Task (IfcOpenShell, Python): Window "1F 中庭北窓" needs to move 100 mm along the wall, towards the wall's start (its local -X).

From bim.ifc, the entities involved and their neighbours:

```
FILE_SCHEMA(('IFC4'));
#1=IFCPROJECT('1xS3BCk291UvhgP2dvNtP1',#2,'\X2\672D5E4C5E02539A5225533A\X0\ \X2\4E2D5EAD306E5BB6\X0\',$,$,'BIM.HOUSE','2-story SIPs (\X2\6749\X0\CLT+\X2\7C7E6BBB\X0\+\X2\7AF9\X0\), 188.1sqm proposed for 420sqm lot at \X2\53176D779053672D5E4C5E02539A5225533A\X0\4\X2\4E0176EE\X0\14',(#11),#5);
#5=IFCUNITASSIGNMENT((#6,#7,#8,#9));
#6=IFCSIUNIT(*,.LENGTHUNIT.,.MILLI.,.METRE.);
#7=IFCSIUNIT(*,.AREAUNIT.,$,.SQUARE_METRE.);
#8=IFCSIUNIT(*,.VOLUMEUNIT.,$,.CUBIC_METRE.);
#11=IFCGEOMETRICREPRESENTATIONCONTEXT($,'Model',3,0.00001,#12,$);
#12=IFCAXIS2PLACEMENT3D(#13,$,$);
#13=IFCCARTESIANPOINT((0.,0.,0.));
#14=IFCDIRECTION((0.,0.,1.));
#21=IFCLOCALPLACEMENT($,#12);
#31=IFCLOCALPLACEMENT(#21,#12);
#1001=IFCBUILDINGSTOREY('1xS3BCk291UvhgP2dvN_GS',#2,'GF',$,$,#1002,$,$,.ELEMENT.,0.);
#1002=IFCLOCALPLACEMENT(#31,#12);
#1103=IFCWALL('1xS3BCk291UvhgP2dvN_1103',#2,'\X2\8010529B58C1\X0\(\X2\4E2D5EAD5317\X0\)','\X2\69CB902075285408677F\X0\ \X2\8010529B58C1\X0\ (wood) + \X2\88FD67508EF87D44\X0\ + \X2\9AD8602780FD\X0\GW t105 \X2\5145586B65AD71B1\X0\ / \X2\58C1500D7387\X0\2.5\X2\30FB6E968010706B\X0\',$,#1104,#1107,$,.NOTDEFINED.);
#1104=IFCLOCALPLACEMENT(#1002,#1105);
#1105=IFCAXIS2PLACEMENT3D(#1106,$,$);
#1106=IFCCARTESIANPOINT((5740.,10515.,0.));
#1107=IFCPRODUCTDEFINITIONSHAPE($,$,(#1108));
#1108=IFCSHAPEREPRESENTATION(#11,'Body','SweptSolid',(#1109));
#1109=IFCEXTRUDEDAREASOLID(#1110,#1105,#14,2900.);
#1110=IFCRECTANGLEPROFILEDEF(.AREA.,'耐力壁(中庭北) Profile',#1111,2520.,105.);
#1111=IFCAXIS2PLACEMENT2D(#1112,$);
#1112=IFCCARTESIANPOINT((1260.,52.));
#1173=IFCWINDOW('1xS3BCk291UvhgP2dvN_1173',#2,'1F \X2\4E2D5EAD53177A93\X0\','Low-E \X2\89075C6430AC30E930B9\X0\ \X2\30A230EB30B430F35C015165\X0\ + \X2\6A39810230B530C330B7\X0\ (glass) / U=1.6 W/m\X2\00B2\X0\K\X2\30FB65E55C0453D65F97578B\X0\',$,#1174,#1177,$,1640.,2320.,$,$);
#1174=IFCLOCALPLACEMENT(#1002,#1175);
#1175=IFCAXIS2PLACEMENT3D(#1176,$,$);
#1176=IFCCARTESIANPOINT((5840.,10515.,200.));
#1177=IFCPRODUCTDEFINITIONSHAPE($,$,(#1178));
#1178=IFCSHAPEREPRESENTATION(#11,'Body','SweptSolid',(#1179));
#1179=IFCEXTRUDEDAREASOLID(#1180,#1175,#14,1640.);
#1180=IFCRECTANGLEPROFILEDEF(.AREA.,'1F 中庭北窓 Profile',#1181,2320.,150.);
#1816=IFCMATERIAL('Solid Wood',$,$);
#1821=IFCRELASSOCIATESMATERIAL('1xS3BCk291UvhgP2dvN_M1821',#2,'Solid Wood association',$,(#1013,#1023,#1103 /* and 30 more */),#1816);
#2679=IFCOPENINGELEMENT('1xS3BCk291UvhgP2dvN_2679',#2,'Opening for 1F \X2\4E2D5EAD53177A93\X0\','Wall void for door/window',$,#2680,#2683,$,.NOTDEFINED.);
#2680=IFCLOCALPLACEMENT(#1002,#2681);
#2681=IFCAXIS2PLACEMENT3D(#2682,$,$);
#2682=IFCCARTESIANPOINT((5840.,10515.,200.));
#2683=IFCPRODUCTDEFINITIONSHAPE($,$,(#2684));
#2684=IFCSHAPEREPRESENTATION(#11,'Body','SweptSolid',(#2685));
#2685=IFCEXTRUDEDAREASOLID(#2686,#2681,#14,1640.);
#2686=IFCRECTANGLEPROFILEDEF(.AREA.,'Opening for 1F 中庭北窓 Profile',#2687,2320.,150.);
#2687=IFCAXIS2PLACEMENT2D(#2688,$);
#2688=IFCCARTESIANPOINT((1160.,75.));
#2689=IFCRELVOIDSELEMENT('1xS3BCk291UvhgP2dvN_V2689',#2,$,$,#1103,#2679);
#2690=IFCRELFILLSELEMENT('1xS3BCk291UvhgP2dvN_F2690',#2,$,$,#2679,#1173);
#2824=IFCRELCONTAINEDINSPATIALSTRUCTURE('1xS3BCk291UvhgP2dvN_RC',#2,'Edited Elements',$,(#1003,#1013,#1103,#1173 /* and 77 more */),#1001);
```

```python
import ifcopenshell
import ifcopenshell.api.geometry
import ifcopenshell.util.placement

model = ifcopenshell.open("bim.ifc")

window = model.by_guid("1xS3BCk291UvhgP2dvN_1173")
opening = window.FillsVoids[0].RelatingOpeningElement
wall = opening.VoidsElements[0].RelatingBuildingElement

wall_matrix = ifcopenshell.util.placement.get_local_placement(wall.ObjectPlacement)
shift = wall_matrix[:3, 0] * -100.0
before = ifcopenshell.util.placement.get_local_placement(window.ObjectPlacement)[:3, 3].copy()

# The window is not placed relative to its opening, so move both.
for product in (opening, window):
    matrix = ifcopenshell.util.placement.get_local_placement(product.ObjectPlacement)
    matrix[:3, 3] += shift
    ifcopenshell.api.geometry.edit_object_placement(model, product=product, matrix=matrix, is_si=False)

after = ifcopenshell.util.placement.get_local_placement(window.ObjectPlacement)[:3, 3]
print("window moved by", (after - before).round(3) + 0.0)

model.write("bim_edited.ifc")
```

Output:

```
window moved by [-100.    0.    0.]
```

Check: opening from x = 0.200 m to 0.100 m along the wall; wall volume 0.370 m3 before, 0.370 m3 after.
